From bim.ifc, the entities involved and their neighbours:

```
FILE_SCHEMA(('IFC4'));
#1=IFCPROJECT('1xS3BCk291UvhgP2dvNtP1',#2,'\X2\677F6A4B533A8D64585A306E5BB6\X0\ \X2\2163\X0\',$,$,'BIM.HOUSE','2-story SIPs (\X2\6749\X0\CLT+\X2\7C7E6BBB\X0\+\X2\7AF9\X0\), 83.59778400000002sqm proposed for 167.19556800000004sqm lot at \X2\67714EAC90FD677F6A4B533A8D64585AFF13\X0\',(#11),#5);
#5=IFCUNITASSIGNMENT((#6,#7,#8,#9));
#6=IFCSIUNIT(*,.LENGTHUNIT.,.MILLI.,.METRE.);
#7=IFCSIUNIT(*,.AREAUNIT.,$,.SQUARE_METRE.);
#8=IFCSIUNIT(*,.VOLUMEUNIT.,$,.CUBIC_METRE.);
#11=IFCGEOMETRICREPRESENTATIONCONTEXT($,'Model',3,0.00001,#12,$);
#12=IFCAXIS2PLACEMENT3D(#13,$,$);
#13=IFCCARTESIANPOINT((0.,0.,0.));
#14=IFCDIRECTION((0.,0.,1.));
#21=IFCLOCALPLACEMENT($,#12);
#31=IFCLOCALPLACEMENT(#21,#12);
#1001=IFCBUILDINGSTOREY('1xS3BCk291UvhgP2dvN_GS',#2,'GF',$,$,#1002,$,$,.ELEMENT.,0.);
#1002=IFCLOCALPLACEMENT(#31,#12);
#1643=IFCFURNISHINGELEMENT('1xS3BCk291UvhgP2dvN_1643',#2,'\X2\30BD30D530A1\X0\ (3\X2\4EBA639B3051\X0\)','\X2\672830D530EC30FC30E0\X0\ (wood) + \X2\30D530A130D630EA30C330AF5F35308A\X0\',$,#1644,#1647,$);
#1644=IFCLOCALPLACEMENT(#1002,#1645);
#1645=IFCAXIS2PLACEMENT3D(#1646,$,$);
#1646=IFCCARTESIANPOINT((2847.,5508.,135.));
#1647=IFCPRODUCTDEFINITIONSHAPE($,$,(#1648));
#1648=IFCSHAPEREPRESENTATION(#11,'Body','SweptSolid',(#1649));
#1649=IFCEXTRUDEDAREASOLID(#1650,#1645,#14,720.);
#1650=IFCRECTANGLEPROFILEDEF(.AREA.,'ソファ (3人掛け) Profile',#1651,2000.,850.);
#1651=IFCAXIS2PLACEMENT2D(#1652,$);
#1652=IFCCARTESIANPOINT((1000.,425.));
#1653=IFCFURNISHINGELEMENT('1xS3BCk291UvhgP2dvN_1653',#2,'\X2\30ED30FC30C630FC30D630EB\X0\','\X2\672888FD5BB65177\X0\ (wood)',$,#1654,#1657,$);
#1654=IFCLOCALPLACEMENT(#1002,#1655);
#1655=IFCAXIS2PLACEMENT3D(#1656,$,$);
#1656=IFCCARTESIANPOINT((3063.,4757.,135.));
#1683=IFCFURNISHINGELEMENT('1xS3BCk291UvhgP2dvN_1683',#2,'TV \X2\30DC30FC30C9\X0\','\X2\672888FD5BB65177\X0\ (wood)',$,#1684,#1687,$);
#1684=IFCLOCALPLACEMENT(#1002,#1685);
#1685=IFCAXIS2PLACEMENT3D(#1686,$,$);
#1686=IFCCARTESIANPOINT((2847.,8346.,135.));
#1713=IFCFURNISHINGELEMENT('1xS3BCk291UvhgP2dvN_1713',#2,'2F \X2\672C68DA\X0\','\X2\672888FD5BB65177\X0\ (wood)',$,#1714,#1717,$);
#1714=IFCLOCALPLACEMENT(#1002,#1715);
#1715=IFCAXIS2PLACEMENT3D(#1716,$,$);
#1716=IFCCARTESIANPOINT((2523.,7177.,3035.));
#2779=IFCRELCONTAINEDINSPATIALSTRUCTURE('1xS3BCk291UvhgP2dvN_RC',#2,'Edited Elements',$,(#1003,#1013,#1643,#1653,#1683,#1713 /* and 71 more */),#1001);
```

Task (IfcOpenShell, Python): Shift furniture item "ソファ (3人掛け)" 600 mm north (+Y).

```python
import ifcopenshell
import ifcopenshell.api.geometry
import ifcopenshell.util.placement
import ifcopenshell.util.unit

model = ifcopenshell.open("bim.ifc")
unit_scale = ifcopenshell.util.unit.calculate_unit_scale(model)

item = model.by_id(1643)
matrix = ifcopenshell.util.placement.get_local_placement(item.ObjectPlacement)
matrix[1, 3] += 0.6 / unit_scale
ifcopenshell.api.geometry.edit_object_placement(model, product=item, matrix=matrix, is_si=False)

print(ifcopenshell.util.placement.get_local_placement(item.ObjectPlacement).round(3) + 0.0)

model.write("bim-out.ifc")
```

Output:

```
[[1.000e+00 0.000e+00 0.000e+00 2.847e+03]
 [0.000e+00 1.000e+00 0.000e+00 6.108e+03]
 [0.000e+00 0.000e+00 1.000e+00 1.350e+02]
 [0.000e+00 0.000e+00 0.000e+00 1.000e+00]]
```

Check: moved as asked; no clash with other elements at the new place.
